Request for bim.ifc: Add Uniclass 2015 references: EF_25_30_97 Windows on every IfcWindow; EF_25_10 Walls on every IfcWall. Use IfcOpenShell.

First a look at what the model holds.

```python
import ifcopenshell

model = ifcopenshell.open("bim.ifc")
print(model.schema)
print("classifications:", [c.Name for c in model.by_type("IfcClassification")])
for ifc_class in ("IfcDoor", "IfcRoof", "IfcStair", "IfcWall", "IfcWindow"):
    print(ifc_class, len(model.by_type(ifc_class)))
```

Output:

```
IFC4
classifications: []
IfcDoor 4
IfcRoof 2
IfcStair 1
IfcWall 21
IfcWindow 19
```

```python
import ifcopenshell
import ifcopenshell.api.classification

model = ifcopenshell.open("bim.ifc")

system = ifcopenshell.api.classification.add_classification(model, classification="Uniclass 2015")

codes = {
    "IfcWindow": ("EF_25_30_97", "Windows"),
    "IfcWall": ("EF_25_10", "Walls"),
}
for ifc_class, (code, name) in codes.items():
    products = model.by_type(ifc_class)
    ifcopenshell.api.classification.add_reference(
        model, products=products, classification=system, identification=code, name=name
    )
    print(code, len(products))

model.write("bim-out.ifc")
```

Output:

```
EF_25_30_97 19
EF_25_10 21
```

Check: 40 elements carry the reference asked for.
